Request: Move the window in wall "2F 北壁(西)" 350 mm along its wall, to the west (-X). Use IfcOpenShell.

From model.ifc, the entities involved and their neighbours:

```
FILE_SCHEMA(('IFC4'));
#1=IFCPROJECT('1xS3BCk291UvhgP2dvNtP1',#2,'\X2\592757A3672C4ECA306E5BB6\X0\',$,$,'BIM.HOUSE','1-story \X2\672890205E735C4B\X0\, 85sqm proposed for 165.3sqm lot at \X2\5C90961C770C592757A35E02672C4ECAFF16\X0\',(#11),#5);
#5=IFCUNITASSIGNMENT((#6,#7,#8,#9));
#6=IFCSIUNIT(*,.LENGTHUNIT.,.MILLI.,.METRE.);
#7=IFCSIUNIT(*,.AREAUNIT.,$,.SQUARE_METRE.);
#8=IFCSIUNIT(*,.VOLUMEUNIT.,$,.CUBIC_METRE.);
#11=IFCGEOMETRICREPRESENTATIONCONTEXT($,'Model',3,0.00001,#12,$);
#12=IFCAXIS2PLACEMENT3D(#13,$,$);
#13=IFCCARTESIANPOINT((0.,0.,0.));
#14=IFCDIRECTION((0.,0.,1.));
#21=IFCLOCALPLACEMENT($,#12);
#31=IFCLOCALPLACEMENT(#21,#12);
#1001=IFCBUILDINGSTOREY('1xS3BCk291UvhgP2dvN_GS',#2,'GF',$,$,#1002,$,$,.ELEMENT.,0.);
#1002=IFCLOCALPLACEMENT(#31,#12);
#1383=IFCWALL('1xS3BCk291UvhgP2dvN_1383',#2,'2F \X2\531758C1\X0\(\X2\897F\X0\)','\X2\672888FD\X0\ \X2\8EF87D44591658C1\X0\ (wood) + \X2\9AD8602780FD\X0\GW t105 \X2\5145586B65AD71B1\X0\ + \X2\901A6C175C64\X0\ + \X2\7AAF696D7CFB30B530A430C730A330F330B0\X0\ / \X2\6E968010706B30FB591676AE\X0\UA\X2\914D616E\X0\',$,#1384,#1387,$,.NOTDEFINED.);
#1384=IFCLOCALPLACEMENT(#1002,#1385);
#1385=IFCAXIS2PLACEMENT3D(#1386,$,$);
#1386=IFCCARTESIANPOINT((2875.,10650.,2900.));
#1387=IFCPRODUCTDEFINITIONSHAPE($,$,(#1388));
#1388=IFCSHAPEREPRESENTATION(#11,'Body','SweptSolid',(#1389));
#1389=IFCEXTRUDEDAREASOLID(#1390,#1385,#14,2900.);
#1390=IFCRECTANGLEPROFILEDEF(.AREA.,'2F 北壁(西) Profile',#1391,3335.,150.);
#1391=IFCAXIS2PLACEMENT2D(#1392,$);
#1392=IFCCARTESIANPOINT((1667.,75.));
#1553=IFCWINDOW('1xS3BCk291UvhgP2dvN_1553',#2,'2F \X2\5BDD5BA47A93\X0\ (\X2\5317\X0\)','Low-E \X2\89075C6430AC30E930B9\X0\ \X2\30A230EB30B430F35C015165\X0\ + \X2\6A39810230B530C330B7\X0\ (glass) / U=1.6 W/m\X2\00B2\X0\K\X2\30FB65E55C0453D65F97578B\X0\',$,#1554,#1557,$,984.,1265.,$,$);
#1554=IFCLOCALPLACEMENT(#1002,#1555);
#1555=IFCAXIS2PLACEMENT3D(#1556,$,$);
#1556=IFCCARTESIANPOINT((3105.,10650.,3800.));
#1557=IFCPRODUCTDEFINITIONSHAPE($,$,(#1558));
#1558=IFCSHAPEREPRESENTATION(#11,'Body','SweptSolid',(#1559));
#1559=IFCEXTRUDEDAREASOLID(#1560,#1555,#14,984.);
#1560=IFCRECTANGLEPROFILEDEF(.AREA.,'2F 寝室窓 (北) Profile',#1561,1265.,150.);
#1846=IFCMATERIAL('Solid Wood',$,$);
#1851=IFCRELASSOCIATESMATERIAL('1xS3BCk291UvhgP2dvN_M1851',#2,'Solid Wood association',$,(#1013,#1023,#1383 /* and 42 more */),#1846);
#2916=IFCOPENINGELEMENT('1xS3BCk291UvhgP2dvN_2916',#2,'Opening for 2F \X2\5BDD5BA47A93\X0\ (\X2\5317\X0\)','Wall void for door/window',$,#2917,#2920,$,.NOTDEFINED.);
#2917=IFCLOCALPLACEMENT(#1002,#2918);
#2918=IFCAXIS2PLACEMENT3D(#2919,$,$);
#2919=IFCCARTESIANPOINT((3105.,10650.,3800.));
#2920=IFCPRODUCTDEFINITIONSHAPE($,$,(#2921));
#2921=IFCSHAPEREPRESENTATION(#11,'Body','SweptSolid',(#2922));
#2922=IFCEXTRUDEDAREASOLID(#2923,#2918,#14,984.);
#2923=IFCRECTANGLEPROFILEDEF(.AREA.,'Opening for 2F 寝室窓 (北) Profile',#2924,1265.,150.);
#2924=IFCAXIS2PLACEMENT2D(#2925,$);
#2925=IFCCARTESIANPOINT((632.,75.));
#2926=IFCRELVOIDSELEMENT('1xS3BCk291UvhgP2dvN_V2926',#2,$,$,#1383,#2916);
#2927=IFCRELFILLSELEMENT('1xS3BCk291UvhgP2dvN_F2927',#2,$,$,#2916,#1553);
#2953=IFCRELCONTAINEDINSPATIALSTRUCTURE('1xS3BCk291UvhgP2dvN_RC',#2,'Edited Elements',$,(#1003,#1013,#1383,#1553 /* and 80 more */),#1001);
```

```python
import ifcopenshell
import ifcopenshell.api.geometry
import ifcopenshell.util.placement
import ifcopenshell.util.unit

model = ifcopenshell.open("model.ifc")
unit_scale = ifcopenshell.util.unit.calculate_unit_scale(model)

window = model.by_id(1553)
opening = window.FillsVoids[0].RelatingOpeningElement
wall = opening.VoidsElements[0].RelatingBuildingElement

wall_matrix = ifcopenshell.util.placement.get_local_placement(wall.ObjectPlacement)
shift = wall_matrix[:3, 0] * -0.35 / unit_scale
before = ifcopenshell.util.placement.get_local_placement(window.ObjectPlacement)[:3, 3].copy()

# The window is not placed relative to its opening, so move both.
for product in (opening, window):
    matrix = ifcopenshell.util.placement.get_local_placement(product.ObjectPlacement)
    matrix[:3, 3] += shift
    ifcopenshell.api.geometry.edit_object_placement(model, product=product, matrix=matrix, is_si=False)

after = ifcopenshell.util.placement.get_local_placement(window.ObjectPlacement)[:3, 3]
print("window moved by", (after - before).round(3) + 0.0)

model.write("model-out.ifc")
```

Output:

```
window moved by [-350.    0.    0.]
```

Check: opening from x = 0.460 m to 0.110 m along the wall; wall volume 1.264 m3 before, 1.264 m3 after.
